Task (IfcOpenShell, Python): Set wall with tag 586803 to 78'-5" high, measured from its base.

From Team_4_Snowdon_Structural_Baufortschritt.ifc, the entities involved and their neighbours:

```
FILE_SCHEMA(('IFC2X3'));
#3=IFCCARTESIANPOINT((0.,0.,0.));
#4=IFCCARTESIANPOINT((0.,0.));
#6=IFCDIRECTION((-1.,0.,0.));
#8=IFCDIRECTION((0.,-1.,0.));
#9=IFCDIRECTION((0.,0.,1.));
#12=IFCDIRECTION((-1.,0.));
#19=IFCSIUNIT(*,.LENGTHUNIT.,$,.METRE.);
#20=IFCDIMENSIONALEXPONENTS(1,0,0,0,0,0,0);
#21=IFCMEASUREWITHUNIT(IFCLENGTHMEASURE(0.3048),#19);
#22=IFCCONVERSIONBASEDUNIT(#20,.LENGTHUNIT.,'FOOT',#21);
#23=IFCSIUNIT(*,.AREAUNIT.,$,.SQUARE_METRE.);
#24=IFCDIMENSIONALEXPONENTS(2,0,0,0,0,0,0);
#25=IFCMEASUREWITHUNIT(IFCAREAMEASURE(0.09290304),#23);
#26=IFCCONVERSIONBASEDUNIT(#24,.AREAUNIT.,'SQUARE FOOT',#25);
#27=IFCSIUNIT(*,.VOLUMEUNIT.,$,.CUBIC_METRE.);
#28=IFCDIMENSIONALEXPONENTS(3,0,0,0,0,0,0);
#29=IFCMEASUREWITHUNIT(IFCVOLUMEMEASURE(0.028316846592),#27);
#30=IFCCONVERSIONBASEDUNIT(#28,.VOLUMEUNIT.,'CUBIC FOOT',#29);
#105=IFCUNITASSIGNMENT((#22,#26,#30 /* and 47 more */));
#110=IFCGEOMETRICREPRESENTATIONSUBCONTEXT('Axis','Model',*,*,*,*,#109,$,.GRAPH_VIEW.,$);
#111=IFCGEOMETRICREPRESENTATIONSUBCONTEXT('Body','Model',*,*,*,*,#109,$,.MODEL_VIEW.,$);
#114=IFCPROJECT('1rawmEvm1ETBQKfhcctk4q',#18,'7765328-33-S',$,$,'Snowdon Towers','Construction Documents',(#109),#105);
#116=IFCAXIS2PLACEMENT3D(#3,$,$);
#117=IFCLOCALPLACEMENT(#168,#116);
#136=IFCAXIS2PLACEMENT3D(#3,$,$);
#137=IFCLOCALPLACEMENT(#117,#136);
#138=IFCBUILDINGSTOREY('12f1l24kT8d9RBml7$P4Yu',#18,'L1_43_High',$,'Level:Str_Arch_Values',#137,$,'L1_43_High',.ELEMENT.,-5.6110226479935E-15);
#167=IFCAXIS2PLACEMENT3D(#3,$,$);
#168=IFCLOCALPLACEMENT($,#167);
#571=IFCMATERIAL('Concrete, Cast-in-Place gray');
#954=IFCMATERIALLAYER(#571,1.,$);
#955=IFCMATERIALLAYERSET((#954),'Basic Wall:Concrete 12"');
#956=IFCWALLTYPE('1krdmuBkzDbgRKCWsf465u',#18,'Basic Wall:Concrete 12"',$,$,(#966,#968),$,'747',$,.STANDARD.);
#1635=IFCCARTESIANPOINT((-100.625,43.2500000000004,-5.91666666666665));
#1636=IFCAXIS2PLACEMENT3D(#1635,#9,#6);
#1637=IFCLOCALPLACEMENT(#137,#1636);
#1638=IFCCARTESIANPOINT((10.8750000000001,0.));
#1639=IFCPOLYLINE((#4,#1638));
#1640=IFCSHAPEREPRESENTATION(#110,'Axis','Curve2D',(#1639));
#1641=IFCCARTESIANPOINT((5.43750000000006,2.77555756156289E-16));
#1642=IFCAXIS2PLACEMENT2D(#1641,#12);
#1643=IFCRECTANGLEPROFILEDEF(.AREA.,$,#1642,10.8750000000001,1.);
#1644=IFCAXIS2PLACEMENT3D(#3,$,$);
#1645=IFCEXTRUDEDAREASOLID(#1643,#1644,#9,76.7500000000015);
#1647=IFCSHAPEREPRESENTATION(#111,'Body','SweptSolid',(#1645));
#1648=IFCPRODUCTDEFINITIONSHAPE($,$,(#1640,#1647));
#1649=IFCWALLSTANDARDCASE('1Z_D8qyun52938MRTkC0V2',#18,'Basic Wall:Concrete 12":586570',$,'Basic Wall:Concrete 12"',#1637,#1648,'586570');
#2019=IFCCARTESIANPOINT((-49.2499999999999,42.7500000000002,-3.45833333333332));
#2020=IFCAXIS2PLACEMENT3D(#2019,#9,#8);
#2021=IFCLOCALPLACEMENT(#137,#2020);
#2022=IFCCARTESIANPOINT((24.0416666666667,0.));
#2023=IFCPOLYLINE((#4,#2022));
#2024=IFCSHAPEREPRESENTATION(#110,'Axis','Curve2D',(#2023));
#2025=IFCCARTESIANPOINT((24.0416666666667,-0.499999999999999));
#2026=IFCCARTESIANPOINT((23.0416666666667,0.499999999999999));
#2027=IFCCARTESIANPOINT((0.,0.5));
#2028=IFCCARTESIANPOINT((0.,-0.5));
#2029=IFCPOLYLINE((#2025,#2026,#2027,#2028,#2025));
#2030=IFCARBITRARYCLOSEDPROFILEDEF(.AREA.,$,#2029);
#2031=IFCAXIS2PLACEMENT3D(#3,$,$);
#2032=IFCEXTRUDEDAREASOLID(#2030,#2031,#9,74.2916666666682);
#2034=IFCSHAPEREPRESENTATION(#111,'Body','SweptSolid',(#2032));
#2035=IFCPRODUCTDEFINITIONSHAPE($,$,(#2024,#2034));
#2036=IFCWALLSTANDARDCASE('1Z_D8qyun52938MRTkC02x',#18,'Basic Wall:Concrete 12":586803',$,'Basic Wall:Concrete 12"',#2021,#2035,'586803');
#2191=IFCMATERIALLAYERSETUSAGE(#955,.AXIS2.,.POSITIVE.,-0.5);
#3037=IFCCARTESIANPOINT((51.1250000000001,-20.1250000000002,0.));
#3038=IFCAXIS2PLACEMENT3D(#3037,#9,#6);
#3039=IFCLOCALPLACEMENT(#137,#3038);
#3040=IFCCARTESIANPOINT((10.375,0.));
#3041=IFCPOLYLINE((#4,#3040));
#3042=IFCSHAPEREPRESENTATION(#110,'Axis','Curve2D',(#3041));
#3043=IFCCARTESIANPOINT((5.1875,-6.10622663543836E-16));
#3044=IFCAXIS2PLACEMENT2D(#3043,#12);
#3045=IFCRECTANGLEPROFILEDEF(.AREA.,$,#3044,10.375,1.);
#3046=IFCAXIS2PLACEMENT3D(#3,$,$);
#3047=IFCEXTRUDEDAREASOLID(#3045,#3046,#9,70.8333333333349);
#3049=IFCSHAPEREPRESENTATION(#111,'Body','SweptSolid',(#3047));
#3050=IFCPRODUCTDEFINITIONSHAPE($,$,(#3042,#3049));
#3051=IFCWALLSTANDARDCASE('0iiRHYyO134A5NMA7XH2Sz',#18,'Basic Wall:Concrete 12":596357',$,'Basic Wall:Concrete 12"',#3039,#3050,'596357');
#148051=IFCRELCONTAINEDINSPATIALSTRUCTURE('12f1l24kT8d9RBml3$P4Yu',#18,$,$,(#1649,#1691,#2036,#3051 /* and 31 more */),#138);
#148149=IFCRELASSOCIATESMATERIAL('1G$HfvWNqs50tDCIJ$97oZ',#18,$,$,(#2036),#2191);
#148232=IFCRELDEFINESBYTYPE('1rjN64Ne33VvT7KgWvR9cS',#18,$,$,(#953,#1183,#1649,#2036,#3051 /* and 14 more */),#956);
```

```python
import ifcopenshell
import ifcopenshell.geom
import ifcopenshell.util.representation
import ifcopenshell.util.shape
import ifcopenshell.util.unit

model = ifcopenshell.open("Team_4_Snowdon_Structural_Baufortschritt.ifc")
unit_scale = ifcopenshell.util.unit.calculate_unit_scale(model)
settings = ifcopenshell.geom.settings()


def volume(element):
    """Net volume in cubic metres, openings subtracted."""
    shape = ifcopenshell.geom.create_shape(settings, element)
    return ifcopenshell.util.shape.get_volume(shape.geometry)


wall = model.by_id(2036)
before = volume(wall)

body = ifcopenshell.util.representation.get_representation(wall, "Model", "Body")
solid = body.Items[0]
old_height = solid.Depth
solid.Depth = 941 * 0.0254 / unit_scale
after = volume(wall)

print(f"height {old_height:g} -> {solid.Depth:g}, volume {before:.3f} -> {after:.3f} m3")

model.write("Team_4_Snowdon_Structural_Baufortschritt_edited.ifc")
```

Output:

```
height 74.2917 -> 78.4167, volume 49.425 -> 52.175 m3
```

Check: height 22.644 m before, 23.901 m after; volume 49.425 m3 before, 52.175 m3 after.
